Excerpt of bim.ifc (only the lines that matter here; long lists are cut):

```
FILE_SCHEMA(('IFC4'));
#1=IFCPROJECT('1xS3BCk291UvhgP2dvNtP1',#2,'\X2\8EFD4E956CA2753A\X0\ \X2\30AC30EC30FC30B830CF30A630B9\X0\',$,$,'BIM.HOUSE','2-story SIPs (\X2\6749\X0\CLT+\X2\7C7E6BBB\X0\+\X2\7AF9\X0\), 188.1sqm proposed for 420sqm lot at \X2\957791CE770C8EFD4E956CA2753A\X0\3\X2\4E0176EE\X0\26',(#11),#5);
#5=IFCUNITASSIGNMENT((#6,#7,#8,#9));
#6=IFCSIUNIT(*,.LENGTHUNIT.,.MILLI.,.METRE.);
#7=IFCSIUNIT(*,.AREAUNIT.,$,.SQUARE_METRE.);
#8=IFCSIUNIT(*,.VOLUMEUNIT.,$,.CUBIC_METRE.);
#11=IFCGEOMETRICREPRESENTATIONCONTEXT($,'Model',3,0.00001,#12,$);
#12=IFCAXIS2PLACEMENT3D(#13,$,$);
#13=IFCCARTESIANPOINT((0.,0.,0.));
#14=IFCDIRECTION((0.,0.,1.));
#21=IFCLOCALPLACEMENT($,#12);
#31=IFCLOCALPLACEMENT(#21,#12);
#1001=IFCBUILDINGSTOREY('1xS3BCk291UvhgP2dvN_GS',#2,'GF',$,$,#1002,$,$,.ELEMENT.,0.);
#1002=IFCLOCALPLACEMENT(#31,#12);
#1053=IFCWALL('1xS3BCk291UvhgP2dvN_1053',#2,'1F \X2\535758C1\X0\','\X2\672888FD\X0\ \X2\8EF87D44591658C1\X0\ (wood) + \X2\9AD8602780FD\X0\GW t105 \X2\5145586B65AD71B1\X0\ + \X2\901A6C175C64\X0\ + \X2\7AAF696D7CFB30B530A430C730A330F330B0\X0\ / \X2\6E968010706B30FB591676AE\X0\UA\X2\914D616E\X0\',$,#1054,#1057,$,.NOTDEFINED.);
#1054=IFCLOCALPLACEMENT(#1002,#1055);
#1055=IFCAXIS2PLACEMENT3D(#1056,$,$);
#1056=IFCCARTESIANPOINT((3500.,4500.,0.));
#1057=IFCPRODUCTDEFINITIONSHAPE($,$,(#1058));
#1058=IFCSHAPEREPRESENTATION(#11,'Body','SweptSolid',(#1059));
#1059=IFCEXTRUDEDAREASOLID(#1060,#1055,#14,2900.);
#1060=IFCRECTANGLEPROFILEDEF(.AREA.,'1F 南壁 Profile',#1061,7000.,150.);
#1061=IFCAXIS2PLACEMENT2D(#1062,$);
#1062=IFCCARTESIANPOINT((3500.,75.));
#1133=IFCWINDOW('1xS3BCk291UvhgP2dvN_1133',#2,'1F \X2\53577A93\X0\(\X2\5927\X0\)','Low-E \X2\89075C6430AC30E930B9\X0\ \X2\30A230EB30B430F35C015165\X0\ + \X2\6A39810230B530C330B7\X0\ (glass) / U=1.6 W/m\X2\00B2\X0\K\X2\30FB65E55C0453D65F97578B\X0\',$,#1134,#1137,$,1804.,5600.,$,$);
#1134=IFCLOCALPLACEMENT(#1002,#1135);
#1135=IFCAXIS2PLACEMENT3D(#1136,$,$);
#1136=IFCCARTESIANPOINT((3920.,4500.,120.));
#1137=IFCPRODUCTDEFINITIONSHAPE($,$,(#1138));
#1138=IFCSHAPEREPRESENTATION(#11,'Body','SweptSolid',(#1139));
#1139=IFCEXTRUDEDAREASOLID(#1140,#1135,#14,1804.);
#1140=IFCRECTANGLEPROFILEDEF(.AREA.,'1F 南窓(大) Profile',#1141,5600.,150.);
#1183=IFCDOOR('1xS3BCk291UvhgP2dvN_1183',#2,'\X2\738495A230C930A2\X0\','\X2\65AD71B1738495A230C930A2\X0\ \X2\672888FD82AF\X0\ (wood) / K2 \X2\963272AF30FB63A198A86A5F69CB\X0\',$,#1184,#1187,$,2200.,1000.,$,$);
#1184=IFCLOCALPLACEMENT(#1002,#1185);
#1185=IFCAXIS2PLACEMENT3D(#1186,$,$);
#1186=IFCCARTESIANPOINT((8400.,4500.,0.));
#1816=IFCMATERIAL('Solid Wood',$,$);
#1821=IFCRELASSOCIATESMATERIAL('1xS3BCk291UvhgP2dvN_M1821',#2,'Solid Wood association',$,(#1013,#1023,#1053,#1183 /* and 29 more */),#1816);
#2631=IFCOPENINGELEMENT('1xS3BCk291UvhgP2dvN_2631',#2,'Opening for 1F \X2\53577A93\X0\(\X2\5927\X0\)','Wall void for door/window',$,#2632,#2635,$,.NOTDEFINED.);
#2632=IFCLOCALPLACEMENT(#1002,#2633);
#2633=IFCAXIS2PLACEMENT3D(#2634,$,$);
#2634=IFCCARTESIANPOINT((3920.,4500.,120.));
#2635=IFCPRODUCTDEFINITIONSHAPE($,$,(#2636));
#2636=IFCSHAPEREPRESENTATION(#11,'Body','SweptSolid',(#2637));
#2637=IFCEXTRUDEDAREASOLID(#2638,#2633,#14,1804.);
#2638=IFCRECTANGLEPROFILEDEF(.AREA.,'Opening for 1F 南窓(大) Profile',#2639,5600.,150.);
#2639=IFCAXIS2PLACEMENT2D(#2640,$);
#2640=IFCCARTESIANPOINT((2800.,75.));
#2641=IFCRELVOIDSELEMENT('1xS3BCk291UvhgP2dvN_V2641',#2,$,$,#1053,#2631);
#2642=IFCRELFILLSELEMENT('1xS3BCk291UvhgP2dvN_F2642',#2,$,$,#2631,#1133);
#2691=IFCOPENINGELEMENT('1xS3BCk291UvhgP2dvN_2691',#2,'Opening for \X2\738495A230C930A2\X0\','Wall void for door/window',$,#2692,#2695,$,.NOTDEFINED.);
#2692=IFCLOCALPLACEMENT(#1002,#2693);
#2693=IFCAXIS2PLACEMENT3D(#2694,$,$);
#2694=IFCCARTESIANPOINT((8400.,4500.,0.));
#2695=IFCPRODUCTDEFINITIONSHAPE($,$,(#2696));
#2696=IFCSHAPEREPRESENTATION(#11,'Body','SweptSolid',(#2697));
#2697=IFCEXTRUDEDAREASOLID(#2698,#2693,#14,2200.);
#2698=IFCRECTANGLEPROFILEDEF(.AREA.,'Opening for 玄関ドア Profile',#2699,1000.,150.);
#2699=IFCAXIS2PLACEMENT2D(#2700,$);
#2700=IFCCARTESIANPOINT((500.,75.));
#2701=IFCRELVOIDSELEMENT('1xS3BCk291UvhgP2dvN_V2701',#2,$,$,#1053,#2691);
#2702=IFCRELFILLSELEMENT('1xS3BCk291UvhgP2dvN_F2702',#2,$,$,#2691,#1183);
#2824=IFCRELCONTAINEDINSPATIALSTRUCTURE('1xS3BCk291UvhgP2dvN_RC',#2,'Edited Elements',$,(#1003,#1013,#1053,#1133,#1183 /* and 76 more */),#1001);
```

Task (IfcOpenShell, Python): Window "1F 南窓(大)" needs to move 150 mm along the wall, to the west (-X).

```python
import ifcopenshell
import ifcopenshell.api.geometry
import ifcopenshell.util.placement
import ifcopenshell.util.unit

model = ifcopenshell.open("bim.ifc")
unit_scale = ifcopenshell.util.unit.calculate_unit_scale(model)

window = model.by_id(1133)
opening = window.FillsVoids[0].RelatingOpeningElement
wall = opening.VoidsElements[0].RelatingBuildingElement

wall_matrix = ifcopenshell.util.placement.get_local_placement(wall.ObjectPlacement)
shift = wall_matrix[:3, 0] * -0.15 / unit_scale
before = ifcopenshell.util.placement.get_local_placement(window.ObjectPlacement)[:3, 3].copy()

# The window is not placed relative to its opening, so move both.
for product in (opening, window):
    matrix = ifcopenshell.util.placement.get_local_placement(product.ObjectPlacement)
    matrix[:3, 3] += shift
    ifcopenshell.api.geometry.edit_object_placement(model, product=product, matrix=matrix, is_si=False)

after = ifcopenshell.util.placement.get_local_placement(window.ObjectPlacement)[:3, 3]
print("window moved by", (after - before).round(3) + 0.0)

model.write("bim_edited.ifc")
```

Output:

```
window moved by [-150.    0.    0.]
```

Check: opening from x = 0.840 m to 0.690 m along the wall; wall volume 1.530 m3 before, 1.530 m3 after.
